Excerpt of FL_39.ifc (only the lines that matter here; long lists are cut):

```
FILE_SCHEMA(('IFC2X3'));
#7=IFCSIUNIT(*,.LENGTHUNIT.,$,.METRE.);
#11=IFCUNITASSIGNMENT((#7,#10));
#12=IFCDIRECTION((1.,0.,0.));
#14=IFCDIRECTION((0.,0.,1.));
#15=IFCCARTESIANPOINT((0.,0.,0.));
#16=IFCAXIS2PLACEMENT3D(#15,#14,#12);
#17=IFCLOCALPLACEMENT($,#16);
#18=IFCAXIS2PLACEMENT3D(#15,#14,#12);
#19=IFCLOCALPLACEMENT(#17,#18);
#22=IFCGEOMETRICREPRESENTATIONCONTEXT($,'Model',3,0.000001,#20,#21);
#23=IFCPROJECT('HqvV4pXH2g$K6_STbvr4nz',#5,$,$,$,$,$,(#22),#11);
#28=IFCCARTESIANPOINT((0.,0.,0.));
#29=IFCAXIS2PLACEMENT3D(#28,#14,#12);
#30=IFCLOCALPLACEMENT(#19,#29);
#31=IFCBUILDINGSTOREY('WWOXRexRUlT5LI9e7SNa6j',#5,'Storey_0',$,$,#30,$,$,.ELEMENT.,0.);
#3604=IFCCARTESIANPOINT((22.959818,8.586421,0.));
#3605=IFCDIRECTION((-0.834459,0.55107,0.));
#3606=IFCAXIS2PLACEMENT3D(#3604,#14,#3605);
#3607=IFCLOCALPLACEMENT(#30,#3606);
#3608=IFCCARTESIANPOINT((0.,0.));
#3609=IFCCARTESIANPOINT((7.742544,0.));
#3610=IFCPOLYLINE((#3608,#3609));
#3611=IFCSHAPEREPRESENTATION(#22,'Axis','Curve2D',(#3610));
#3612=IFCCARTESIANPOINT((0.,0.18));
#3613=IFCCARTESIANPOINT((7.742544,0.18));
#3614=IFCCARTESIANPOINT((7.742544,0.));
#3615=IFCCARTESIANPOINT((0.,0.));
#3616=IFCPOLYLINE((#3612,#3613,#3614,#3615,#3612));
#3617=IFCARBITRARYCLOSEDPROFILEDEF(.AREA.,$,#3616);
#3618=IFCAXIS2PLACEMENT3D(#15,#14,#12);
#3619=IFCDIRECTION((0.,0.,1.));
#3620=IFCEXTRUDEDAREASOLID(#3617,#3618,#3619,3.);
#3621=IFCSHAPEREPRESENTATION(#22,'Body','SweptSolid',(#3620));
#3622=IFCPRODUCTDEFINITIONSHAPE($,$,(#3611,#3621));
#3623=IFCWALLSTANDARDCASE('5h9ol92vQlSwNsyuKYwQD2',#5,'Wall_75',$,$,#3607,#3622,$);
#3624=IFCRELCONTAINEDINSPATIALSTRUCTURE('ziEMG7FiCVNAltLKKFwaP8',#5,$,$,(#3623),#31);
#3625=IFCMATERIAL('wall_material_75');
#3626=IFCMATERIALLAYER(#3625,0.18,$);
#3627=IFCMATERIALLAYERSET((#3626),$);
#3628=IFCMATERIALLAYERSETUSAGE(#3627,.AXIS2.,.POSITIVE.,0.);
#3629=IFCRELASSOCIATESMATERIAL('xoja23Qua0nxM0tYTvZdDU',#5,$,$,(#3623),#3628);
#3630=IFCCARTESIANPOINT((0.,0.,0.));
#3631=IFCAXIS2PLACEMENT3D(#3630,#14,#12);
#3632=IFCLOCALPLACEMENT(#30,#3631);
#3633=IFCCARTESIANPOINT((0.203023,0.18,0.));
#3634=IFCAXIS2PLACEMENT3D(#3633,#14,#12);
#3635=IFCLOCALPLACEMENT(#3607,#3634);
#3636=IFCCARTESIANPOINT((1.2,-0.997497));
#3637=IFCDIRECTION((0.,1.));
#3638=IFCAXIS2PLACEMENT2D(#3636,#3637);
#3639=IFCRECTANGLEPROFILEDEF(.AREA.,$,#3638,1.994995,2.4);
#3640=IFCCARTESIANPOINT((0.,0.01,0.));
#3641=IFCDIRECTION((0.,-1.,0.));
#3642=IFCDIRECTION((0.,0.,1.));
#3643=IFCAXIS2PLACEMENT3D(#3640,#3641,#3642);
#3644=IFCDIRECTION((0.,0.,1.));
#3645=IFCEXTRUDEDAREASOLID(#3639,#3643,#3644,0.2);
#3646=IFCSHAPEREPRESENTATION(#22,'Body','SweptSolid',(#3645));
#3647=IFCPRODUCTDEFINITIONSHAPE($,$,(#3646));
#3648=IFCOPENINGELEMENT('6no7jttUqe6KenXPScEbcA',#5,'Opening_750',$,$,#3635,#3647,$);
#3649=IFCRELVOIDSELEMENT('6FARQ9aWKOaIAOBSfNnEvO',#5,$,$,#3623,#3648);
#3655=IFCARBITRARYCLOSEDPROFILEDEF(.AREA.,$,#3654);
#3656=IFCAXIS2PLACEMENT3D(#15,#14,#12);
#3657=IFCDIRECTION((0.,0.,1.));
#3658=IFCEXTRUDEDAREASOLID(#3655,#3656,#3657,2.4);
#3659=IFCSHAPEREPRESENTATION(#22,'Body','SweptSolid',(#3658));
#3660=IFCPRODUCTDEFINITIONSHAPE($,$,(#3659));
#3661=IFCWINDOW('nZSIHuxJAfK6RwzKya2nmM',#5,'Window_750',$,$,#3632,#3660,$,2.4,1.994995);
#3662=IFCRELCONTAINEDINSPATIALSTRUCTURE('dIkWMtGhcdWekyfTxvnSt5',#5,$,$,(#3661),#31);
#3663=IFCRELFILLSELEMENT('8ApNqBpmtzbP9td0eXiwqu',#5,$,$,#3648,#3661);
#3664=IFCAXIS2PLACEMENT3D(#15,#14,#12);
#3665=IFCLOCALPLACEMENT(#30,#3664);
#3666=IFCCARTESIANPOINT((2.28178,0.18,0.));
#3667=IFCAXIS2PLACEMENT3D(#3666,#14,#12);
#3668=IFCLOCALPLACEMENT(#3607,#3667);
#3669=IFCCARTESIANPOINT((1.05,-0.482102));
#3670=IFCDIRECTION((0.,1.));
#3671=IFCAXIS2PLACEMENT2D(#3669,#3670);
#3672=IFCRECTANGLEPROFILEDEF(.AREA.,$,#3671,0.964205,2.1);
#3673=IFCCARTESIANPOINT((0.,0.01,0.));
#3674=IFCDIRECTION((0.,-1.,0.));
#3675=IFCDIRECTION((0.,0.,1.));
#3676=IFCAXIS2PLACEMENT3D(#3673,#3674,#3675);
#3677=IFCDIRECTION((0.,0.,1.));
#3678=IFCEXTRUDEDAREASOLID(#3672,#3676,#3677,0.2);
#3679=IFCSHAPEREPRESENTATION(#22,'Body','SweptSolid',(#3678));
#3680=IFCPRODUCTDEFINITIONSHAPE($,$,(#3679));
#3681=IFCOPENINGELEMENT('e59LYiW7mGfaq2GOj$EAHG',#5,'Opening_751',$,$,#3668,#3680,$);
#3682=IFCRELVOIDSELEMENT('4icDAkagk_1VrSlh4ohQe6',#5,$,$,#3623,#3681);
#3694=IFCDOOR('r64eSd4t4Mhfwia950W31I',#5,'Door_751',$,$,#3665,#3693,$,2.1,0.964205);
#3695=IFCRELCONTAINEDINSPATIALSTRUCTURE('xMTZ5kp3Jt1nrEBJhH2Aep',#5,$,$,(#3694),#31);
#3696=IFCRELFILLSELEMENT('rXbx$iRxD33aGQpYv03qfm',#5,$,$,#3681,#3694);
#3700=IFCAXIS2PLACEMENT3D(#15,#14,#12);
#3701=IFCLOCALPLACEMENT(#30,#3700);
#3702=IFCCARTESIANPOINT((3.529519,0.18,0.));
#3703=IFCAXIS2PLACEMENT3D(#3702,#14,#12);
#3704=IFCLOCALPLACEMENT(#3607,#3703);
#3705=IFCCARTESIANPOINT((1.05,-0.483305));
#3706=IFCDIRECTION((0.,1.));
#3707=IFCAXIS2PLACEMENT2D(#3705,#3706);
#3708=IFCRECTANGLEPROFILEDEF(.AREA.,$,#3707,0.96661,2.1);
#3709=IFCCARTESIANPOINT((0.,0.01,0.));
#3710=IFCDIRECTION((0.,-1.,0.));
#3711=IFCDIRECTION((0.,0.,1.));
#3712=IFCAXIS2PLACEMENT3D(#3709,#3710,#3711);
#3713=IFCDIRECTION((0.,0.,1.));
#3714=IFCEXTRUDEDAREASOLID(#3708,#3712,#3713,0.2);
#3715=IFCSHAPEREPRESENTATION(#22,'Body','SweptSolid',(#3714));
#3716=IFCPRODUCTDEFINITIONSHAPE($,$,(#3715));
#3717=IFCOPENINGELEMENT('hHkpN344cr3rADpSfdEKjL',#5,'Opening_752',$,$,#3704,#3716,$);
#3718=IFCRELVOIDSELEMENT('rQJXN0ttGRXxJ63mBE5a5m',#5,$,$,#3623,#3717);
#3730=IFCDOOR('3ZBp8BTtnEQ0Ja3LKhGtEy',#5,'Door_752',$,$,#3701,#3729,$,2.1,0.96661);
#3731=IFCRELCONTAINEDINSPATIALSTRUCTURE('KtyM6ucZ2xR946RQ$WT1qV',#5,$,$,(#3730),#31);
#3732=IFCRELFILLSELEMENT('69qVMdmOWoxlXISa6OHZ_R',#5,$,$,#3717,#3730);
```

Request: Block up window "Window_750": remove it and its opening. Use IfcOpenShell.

```python
import ifcopenshell
import ifcopenshell.api.feature
import ifcopenshell.api.root
import ifcopenshell.geom
import ifcopenshell.util.shape

model = ifcopenshell.open("FL_39.ifc")
settings = ifcopenshell.geom.settings()


def volume(element):
    """Net volume in cubic metres, openings subtracted."""
    shape = ifcopenshell.geom.create_shape(settings, element)
    return ifcopenshell.util.shape.get_volume(shape.geometry)


window = model.by_guid("nZSIHuxJAfK6RwzKya2nmM")
opening = window.FillsVoids[0].RelatingOpeningElement
wall = opening.VoidsElements[0].RelatingBuildingElement
before = volume(wall)

ifcopenshell.api.root.remove_product(model, product=window)
ifcopenshell.api.feature.remove_feature(model, feature=opening)

after = volume(wall)

print(f"wall volume {before:.3f} -> {after:.3f} m3")

model.write("FL_39_edited.ifc")
```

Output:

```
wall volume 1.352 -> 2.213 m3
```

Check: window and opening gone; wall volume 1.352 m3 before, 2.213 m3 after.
